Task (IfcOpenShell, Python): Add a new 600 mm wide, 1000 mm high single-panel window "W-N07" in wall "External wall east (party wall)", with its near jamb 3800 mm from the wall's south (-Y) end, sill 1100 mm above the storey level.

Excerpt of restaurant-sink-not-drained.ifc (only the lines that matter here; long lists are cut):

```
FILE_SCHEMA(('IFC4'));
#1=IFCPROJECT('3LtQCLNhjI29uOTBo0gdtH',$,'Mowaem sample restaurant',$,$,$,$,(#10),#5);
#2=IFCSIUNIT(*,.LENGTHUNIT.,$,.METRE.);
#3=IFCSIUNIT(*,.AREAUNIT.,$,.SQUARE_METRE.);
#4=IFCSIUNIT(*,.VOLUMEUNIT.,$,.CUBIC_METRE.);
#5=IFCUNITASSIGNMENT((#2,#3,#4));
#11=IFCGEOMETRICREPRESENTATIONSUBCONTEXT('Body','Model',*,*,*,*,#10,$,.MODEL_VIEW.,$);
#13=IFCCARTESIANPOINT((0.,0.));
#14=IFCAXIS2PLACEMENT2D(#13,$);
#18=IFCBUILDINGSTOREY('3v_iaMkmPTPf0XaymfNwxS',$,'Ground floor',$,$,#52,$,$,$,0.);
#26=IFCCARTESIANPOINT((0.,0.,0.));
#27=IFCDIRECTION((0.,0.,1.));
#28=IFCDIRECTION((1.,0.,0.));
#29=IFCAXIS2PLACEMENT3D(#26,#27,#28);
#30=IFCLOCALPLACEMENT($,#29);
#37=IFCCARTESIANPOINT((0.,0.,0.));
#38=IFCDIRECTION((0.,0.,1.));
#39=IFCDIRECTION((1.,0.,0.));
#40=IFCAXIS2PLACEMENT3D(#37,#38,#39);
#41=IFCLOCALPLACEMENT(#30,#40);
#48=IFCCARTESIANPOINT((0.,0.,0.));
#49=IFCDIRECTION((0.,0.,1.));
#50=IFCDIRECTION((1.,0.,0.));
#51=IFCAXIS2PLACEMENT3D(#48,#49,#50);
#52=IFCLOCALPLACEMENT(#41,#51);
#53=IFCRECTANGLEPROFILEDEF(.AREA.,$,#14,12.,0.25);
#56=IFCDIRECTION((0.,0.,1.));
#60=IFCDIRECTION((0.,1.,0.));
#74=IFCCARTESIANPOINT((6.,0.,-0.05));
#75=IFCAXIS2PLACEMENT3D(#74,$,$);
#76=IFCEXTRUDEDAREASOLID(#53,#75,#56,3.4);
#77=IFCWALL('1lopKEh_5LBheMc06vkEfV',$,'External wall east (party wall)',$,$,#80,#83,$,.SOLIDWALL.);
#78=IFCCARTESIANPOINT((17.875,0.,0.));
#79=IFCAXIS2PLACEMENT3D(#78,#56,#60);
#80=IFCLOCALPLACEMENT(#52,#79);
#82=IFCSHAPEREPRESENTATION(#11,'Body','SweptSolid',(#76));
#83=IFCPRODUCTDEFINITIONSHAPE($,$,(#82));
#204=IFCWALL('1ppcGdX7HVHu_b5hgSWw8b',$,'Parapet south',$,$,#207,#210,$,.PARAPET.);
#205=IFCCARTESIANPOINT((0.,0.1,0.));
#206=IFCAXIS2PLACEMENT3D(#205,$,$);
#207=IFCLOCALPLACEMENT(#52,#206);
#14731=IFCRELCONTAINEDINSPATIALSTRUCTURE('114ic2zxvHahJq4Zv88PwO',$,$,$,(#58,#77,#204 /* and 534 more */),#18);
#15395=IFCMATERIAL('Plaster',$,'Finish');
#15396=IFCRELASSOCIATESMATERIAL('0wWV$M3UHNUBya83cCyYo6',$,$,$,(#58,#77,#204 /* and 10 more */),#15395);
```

```python
import numpy as np
import ifcopenshell
import ifcopenshell.api.feature
import ifcopenshell.api.geometry
import ifcopenshell.api.root
import ifcopenshell.api.spatial
import ifcopenshell.geom
import ifcopenshell.util.element
import ifcopenshell.util.placement
import ifcopenshell.util.representation
import ifcopenshell.util.shape
import ifcopenshell.util.unit

model = ifcopenshell.open("restaurant-sink-not-drained.ifc")
unit_scale = ifcopenshell.util.unit.calculate_unit_scale(model)
settings = ifcopenshell.geom.settings()


def volume(element):
    """Net volume in cubic metres, openings subtracted."""
    shape = ifcopenshell.geom.create_shape(settings, element)
    return ifcopenshell.util.shape.get_volume(shape.geometry)


wall = model.by_guid("1lopKEh_5LBheMc06vkEfV")
storey = ifcopenshell.util.element.get_container(wall, ifc_class="IfcBuildingStorey")
context = ifcopenshell.util.representation.get_context(model, "Model", "Body", "MODEL_VIEW")
before = volume(wall)

width, height, from_end, sill = 0.6, 1, 3.8, 1.1  # metres

# The wall runs along its own X axis, and the end named is its -X end.
wall_shape = ifcopenshell.geom.create_shape(settings, wall)
x, y, z = ifcopenshell.util.shape.get_vertices(wall_shape.geometry).T
start = x.min() + from_end
face, thickness = float(y.min()), float(y.max() - y.min())
wall_matrix = ifcopenshell.util.placement.get_local_placement(wall.ObjectPlacement)
level = ifcopenshell.util.placement.get_local_placement(storey.ObjectPlacement)[2, 3]


def in_wall(x, y):
    """Placement at x, y metres in the wall's axes, at sill height."""
    matrix = wall_matrix.copy()
    matrix[:, 3] = wall_matrix @ np.array([x / unit_scale, y / unit_scale, 0.0, 1.0])
    matrix[2, 3] = level + sill / unit_scale
    return matrix


# Opening: a box that overshoots both wall faces by 50 mm.
opening = ifcopenshell.api.root.create_entity(model, ifc_class="IfcOpeningElement", predefined_type="OPENING")
box = ifcopenshell.api.geometry.add_wall_representation(
    model, context=context, length=width, height=height, thickness=thickness + 0.1
)
ifcopenshell.api.geometry.assign_representation(model, product=opening, representation=box)
ifcopenshell.api.geometry.edit_object_placement(model, product=opening, matrix=in_wall(start, face - 0.05), is_si=False)
ifcopenshell.api.feature.add_feature(model, feature=opening, element=wall)

window = ifcopenshell.api.root.create_entity(model, ifc_class="IfcWindow", name="W-N07", predefined_type="WINDOW")
window.OverallWidth, window.OverallHeight = width / unit_scale, height / unit_scale
window.PartitioningType = "SINGLE_PANEL"
body = ifcopenshell.api.geometry.add_window_representation(
    model,
    context=context,
    overall_width=window.OverallWidth,
    overall_height=window.OverallHeight,
    partition_type="SINGLE_PANEL",
)
ifcopenshell.api.geometry.assign_representation(model, product=window, representation=body)
ifcopenshell.api.spatial.assign_container(model, products=[window], relating_structure=storey)
ifcopenshell.api.feature.add_filling(model, opening=opening, element=window)

# Centre the window in the wall's thickness.
ifcopenshell.api.geometry.edit_object_placement(model, product=window, matrix=in_wall(start, face), is_si=False)
window_shape = ifcopenshell.geom.create_shape(settings, window)
depth = ifcopenshell.util.shape.get_vertices(window_shape.geometry)[:, 1]
offset = face + thickness / 2 - (depth.min() + depth.max()) / 2
ifcopenshell.api.geometry.edit_object_placement(model, product=window, matrix=in_wall(start, offset), is_si=False)

after = volume(wall)

print(f"wall volume {before:.3f} -> {after:.3f} m3")

model.write("restaurant-sink-not-drained_edited.ifc")
```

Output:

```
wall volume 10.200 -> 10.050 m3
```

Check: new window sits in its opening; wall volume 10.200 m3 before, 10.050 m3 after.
